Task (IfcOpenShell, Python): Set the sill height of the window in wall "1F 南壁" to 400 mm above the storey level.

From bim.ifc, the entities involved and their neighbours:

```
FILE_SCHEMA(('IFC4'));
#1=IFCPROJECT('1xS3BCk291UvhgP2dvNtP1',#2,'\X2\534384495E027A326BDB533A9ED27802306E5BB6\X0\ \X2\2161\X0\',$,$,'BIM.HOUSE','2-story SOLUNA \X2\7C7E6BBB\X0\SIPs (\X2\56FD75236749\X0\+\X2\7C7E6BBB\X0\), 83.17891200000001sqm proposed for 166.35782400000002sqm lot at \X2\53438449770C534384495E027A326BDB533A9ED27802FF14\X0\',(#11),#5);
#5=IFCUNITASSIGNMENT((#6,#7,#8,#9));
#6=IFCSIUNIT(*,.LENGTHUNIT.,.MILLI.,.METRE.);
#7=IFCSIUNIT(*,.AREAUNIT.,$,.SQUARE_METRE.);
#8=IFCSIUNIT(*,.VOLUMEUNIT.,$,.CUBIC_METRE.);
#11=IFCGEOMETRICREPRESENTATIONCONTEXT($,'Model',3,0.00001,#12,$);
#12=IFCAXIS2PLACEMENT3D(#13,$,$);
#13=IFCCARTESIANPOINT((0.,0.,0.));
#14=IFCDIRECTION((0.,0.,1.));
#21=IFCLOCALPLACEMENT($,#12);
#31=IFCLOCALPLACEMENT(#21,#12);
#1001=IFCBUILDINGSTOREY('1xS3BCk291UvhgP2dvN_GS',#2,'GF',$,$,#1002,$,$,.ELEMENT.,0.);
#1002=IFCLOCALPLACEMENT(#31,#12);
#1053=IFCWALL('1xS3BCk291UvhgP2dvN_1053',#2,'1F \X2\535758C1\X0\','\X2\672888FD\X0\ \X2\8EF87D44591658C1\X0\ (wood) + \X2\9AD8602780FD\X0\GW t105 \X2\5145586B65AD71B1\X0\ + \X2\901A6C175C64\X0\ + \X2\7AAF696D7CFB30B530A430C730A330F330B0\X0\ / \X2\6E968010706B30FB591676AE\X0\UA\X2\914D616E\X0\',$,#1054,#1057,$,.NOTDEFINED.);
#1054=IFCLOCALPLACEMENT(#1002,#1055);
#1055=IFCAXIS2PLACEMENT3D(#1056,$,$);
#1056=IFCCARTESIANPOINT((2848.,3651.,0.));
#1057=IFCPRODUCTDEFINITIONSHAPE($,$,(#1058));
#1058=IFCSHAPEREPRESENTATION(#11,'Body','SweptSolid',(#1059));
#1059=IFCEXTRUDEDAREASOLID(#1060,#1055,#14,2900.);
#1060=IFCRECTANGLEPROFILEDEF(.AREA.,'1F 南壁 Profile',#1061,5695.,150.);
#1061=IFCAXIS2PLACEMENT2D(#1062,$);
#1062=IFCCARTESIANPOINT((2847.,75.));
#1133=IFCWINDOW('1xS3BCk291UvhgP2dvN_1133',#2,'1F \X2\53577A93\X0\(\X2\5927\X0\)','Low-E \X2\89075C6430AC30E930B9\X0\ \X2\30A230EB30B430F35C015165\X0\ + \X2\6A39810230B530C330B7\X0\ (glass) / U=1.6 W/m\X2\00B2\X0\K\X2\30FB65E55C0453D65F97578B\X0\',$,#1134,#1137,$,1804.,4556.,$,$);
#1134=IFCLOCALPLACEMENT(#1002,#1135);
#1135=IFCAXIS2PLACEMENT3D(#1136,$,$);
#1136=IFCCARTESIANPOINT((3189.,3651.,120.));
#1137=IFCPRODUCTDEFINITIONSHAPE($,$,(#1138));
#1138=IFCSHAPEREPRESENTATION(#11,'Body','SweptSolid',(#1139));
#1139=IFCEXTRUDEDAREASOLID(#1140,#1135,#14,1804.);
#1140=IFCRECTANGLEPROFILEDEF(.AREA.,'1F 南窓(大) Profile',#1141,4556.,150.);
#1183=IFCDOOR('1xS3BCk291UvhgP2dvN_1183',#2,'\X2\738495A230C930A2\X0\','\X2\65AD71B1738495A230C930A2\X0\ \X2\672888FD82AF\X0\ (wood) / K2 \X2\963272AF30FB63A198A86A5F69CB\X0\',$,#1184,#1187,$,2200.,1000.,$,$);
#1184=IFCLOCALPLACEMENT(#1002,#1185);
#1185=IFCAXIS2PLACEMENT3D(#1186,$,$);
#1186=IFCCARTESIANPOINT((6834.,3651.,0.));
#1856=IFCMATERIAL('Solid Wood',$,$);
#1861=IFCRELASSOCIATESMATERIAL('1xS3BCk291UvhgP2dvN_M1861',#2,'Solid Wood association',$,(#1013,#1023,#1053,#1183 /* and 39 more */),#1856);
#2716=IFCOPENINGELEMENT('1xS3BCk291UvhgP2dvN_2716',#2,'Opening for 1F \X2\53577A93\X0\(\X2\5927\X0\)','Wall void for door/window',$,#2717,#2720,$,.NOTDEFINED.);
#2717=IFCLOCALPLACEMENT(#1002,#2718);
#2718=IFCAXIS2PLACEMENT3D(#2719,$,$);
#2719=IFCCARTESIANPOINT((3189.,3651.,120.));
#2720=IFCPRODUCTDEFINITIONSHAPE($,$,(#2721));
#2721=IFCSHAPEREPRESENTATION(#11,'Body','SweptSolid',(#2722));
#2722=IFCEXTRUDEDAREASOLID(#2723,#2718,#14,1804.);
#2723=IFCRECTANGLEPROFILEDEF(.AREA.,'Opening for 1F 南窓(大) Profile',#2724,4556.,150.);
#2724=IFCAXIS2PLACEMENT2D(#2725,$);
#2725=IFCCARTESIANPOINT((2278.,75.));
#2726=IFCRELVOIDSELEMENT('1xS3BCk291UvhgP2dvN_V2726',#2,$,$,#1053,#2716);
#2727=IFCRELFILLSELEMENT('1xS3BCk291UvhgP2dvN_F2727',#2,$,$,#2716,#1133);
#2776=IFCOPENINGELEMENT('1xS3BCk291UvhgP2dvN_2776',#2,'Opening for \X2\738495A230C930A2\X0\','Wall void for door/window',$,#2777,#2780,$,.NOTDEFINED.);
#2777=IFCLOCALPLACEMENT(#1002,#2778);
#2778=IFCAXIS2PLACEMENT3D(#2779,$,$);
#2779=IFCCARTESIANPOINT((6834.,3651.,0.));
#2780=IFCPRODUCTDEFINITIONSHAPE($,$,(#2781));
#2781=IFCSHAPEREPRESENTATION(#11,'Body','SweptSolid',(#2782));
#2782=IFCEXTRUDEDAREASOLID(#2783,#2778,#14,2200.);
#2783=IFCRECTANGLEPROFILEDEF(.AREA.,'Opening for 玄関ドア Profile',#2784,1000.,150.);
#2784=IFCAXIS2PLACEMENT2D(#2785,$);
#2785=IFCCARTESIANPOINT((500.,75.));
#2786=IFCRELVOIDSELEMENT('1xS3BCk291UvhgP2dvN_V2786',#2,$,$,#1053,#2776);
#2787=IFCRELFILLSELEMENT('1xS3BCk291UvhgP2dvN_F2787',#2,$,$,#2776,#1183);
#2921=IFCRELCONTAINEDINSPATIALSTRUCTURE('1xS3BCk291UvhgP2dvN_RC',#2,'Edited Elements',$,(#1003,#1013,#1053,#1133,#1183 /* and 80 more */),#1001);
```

```python
import numpy as np
import ifcopenshell
import ifcopenshell.api.geometry
import ifcopenshell.geom
import ifcopenshell.util.element
import ifcopenshell.util.placement
import ifcopenshell.util.shape
import ifcopenshell.util.unit

model = ifcopenshell.open("bim.ifc")
unit_scale = ifcopenshell.util.unit.calculate_unit_scale(model)

window = model.by_id(1133)
opening = window.FillsVoids[0].RelatingOpeningElement
storey = ifcopenshell.util.element.get_container(window, ifc_class="IfcBuildingStorey")
level = ifcopenshell.util.placement.get_local_placement(storey.ObjectPlacement)[2, 3]

# The opening's origin need not be at the sill, so measure its lowest point.
shape = ifcopenshell.geom.create_shape(ifcopenshell.geom.settings(), opening)
bottom = ifcopenshell.util.shape.get_shape_bottom_elevation(shape, shape.geometry) / unit_scale
dz = level + 0.4 / unit_scale - bottom

shift = np.array([0.0, 0.0, dz])
# The window is not placed relative to its opening, so move both.
for product in (opening, window):
    matrix = ifcopenshell.util.placement.get_local_placement(product.ObjectPlacement)
    matrix[:3, 3] += shift
    ifcopenshell.api.geometry.edit_object_placement(model, product=product, matrix=matrix, is_si=False)

print(f"moved by {dz * unit_scale:+.3f} m")

model.write("bim_updated.ifc")
```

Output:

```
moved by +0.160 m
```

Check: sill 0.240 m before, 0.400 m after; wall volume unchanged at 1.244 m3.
